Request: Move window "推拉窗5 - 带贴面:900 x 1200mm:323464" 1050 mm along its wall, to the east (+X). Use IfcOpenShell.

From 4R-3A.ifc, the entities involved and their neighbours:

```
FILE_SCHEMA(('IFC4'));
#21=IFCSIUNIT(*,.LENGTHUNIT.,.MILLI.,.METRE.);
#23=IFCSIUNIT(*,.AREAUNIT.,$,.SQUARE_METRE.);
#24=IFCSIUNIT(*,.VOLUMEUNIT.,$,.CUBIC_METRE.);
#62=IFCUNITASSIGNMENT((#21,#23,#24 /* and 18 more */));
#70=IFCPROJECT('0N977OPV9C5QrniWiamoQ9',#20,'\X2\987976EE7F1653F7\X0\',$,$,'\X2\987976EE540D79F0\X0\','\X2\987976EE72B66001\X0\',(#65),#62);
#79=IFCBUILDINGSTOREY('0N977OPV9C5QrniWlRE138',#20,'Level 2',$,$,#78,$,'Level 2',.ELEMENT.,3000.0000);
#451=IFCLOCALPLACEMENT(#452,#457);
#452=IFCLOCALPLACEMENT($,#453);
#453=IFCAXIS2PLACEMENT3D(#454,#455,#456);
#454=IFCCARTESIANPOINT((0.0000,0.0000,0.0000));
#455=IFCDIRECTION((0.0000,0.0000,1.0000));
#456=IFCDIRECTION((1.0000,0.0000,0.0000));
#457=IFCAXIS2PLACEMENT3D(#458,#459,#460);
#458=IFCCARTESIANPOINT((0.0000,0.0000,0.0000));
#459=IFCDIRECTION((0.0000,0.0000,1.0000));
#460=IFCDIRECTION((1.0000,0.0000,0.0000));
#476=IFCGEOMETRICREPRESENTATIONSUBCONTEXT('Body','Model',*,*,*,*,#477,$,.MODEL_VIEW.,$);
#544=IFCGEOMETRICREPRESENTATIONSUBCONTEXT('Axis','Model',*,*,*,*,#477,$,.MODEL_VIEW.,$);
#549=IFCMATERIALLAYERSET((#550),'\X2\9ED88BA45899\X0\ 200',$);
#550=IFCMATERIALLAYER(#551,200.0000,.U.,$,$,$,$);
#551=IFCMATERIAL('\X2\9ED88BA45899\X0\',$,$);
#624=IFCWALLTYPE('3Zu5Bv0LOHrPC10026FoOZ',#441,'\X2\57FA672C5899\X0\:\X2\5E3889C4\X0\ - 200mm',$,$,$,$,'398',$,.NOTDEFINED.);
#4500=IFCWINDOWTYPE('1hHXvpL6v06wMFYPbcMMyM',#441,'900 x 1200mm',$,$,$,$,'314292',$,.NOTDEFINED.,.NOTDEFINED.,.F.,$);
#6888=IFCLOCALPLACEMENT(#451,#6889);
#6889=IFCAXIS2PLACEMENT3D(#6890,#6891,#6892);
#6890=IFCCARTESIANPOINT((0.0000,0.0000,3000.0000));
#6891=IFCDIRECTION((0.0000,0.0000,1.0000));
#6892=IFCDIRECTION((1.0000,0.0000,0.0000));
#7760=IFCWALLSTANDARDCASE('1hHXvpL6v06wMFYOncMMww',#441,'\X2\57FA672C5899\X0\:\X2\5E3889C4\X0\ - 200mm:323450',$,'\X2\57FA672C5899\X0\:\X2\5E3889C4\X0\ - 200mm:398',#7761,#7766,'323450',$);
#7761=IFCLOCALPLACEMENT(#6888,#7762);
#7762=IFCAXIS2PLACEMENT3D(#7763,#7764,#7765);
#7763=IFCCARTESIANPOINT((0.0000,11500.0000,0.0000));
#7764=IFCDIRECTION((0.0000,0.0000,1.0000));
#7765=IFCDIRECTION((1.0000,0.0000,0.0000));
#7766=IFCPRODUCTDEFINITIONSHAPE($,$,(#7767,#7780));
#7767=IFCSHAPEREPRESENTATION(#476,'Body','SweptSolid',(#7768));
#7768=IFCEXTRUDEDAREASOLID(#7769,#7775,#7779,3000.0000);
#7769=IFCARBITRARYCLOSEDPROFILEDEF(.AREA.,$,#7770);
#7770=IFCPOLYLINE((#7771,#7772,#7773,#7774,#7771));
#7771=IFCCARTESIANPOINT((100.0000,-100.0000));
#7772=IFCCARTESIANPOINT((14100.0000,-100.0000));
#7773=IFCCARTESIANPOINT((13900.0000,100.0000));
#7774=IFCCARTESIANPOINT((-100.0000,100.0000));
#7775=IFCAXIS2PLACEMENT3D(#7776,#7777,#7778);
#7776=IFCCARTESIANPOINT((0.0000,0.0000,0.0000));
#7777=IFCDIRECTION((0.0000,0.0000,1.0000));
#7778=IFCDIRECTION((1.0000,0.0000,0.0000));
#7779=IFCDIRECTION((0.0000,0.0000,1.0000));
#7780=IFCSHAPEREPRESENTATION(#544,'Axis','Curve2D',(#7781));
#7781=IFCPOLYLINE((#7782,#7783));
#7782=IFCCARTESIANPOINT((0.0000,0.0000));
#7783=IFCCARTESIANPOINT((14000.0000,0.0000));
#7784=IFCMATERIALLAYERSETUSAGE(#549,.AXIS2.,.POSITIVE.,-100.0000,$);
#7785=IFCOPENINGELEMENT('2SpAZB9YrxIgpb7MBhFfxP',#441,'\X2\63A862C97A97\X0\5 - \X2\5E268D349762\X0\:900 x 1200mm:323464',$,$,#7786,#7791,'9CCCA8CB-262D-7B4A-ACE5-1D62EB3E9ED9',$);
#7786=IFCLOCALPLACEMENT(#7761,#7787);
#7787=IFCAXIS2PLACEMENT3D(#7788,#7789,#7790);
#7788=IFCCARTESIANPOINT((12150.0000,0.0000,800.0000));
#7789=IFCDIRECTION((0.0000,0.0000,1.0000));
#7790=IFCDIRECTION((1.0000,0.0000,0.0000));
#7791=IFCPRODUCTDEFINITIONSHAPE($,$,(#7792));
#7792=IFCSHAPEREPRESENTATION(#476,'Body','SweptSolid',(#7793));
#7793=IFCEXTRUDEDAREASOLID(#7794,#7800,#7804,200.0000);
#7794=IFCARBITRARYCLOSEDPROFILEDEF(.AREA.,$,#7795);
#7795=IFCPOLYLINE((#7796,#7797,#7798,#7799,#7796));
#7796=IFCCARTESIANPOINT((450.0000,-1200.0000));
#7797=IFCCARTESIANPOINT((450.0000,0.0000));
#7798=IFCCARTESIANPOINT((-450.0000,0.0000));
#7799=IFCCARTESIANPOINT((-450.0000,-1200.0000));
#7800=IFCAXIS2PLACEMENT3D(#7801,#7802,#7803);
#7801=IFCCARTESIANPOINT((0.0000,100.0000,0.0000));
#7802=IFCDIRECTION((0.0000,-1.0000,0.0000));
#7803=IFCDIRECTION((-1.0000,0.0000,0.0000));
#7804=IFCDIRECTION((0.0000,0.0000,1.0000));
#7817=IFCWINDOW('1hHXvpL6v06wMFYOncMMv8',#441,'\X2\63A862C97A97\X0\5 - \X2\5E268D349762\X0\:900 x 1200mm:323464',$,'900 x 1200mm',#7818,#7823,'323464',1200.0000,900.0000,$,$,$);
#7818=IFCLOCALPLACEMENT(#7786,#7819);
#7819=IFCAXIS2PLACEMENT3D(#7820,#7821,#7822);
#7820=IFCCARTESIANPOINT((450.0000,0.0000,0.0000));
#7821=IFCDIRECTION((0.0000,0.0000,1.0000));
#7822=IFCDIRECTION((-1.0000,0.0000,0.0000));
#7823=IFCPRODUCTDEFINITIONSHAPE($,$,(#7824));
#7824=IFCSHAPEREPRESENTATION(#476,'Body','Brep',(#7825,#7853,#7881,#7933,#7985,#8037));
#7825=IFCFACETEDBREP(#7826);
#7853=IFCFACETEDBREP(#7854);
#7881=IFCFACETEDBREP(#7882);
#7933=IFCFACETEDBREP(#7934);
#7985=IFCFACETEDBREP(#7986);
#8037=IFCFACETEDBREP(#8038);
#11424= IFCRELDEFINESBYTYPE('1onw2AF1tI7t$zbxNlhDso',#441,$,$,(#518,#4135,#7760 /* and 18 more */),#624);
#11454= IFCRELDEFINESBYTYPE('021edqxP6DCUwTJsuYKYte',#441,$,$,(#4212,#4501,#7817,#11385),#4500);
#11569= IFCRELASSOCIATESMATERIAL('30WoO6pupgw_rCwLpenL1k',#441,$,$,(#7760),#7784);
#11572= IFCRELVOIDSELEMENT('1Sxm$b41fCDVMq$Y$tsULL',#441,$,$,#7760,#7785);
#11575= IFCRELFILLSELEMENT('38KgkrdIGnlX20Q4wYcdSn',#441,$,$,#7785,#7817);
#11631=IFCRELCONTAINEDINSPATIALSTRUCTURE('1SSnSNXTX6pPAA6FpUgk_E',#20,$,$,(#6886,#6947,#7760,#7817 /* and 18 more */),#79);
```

```python
import ifcopenshell
import ifcopenshell.api.geometry
import ifcopenshell.util.placement
import ifcopenshell.util.unit

model = ifcopenshell.open("4R-3A.ifc")
unit_scale = ifcopenshell.util.unit.calculate_unit_scale(model)

window = model.by_guid("1hHXvpL6v06wMFYOncMMv8")
opening = window.FillsVoids[0].RelatingOpeningElement
wall = opening.VoidsElements[0].RelatingBuildingElement

wall_matrix = ifcopenshell.util.placement.get_local_placement(wall.ObjectPlacement)
shift = wall_matrix[:3, 0] * 1.05 / unit_scale
before = ifcopenshell.util.placement.get_local_placement(window.ObjectPlacement)[:3, 3].copy()

# The window is placed relative to its opening, so it follows when the opening moves.
matrix = ifcopenshell.util.placement.get_local_placement(opening.ObjectPlacement)
matrix[:3, 3] += shift
ifcopenshell.api.geometry.edit_object_placement(
    model, product=opening, matrix=matrix, is_si=False, should_transform_children=True
)

after = ifcopenshell.util.placement.get_local_placement(window.ObjectPlacement)[:3, 3]
print("window moved by", (after - before).round(3) + 0.0)

model.write("4R-3A_updated.ifc")
```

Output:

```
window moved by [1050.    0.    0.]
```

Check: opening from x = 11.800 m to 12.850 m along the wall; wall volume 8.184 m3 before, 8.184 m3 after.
